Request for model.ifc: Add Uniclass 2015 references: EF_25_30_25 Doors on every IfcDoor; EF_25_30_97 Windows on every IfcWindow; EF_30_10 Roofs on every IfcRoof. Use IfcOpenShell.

First a look at what the model holds.

```python
import ifcopenshell

model = ifcopenshell.open("model.ifc")
print(model.schema)
print("classifications:", [c.Name for c in model.by_type("IfcClassification")])
for ifc_class in ("IfcDoor", "IfcRoof", "IfcStair", "IfcWall", "IfcWindow"):
    print(ifc_class, len(model.by_type(ifc_class)))
```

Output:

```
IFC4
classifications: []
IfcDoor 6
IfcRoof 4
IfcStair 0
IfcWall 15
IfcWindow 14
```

```python
import ifcopenshell
import ifcopenshell.api.classification

model = ifcopenshell.open("model.ifc")

system = ifcopenshell.api.classification.add_classification(model, classification="Uniclass 2015")

codes = {
    "IfcDoor": ("EF_25_30_25", "Doors"),
    "IfcWindow": ("EF_25_30_97", "Windows"),
    "IfcRoof": ("EF_30_10", "Roofs"),
}
for ifc_class, (code, name) in codes.items():
    products = model.by_type(ifc_class)
    ifcopenshell.api.classification.add_reference(
        model, products=products, classification=system, identification=code, name=name
    )
    print(code, len(products))

model.write("model_edited.ifc")
```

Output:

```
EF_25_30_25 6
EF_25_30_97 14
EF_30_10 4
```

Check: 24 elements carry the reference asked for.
